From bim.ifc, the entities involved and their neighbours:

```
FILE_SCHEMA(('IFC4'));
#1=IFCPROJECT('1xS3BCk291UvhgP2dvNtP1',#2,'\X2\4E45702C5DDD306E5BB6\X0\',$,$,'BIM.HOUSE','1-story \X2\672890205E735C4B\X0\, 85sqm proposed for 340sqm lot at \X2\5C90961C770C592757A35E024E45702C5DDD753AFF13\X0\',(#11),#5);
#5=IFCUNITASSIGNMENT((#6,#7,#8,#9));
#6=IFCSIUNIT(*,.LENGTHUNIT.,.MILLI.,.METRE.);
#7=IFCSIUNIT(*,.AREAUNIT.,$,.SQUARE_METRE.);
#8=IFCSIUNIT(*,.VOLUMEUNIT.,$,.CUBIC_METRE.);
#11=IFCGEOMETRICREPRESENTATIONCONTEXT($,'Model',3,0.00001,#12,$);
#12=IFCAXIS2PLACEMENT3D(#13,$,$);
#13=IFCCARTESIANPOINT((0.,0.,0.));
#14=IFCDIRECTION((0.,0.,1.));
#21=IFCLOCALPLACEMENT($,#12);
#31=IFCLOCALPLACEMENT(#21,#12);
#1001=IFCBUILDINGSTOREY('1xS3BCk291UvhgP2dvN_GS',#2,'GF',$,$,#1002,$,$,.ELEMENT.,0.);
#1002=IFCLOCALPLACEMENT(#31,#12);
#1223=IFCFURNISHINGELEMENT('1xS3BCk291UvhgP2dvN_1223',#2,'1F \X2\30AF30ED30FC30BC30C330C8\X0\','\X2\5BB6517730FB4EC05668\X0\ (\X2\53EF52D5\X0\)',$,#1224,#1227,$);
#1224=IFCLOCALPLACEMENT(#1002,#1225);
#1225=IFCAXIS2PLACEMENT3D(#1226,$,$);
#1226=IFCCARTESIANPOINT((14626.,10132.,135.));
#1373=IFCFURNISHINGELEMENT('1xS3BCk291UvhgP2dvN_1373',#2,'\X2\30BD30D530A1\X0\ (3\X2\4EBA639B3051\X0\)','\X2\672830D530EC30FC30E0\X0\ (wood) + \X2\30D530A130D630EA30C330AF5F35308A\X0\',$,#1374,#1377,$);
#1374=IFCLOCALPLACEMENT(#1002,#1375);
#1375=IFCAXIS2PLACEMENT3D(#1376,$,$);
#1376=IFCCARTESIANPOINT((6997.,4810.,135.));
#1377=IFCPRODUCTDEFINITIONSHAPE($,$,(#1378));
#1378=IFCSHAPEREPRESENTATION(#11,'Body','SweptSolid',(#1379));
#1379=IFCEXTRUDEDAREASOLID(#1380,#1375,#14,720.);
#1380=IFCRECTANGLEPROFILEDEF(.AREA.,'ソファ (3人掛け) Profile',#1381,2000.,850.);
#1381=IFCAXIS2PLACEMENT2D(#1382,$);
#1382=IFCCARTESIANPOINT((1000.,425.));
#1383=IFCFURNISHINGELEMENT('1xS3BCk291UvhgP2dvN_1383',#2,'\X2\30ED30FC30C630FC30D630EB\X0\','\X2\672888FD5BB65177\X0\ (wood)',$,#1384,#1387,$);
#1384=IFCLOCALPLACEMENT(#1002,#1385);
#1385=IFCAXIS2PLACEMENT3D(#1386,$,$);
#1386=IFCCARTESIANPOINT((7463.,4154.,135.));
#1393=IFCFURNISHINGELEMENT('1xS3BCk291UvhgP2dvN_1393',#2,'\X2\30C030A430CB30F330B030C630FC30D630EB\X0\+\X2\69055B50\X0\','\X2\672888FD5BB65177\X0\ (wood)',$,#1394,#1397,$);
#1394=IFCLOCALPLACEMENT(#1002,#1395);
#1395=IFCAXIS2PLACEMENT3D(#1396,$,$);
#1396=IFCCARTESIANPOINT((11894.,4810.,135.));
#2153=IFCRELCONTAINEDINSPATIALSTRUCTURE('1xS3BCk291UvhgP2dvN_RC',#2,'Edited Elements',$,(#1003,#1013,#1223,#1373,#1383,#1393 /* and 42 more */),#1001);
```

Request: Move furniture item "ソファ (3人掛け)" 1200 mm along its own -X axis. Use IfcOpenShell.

```python
import ifcopenshell
import ifcopenshell.api.geometry
import ifcopenshell.util.placement
import ifcopenshell.util.unit

model = ifcopenshell.open("bim.ifc")
unit_scale = ifcopenshell.util.unit.calculate_unit_scale(model)

item = model.by_guid("1xS3BCk291UvhgP2dvN_1373")
matrix = ifcopenshell.util.placement.get_local_placement(item.ObjectPlacement)
matrix[:3, 3] -= matrix[:3, 0] * 1.2 / unit_scale
ifcopenshell.api.geometry.edit_object_placement(model, product=item, matrix=matrix, is_si=False)

print(ifcopenshell.util.placement.get_local_placement(item.ObjectPlacement).round(3) + 0.0)

model.write("bim_edited.ifc")
```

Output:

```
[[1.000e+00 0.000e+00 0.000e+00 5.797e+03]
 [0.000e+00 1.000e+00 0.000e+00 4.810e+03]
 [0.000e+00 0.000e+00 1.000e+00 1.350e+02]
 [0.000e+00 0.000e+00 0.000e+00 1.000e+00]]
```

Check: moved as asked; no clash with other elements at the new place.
